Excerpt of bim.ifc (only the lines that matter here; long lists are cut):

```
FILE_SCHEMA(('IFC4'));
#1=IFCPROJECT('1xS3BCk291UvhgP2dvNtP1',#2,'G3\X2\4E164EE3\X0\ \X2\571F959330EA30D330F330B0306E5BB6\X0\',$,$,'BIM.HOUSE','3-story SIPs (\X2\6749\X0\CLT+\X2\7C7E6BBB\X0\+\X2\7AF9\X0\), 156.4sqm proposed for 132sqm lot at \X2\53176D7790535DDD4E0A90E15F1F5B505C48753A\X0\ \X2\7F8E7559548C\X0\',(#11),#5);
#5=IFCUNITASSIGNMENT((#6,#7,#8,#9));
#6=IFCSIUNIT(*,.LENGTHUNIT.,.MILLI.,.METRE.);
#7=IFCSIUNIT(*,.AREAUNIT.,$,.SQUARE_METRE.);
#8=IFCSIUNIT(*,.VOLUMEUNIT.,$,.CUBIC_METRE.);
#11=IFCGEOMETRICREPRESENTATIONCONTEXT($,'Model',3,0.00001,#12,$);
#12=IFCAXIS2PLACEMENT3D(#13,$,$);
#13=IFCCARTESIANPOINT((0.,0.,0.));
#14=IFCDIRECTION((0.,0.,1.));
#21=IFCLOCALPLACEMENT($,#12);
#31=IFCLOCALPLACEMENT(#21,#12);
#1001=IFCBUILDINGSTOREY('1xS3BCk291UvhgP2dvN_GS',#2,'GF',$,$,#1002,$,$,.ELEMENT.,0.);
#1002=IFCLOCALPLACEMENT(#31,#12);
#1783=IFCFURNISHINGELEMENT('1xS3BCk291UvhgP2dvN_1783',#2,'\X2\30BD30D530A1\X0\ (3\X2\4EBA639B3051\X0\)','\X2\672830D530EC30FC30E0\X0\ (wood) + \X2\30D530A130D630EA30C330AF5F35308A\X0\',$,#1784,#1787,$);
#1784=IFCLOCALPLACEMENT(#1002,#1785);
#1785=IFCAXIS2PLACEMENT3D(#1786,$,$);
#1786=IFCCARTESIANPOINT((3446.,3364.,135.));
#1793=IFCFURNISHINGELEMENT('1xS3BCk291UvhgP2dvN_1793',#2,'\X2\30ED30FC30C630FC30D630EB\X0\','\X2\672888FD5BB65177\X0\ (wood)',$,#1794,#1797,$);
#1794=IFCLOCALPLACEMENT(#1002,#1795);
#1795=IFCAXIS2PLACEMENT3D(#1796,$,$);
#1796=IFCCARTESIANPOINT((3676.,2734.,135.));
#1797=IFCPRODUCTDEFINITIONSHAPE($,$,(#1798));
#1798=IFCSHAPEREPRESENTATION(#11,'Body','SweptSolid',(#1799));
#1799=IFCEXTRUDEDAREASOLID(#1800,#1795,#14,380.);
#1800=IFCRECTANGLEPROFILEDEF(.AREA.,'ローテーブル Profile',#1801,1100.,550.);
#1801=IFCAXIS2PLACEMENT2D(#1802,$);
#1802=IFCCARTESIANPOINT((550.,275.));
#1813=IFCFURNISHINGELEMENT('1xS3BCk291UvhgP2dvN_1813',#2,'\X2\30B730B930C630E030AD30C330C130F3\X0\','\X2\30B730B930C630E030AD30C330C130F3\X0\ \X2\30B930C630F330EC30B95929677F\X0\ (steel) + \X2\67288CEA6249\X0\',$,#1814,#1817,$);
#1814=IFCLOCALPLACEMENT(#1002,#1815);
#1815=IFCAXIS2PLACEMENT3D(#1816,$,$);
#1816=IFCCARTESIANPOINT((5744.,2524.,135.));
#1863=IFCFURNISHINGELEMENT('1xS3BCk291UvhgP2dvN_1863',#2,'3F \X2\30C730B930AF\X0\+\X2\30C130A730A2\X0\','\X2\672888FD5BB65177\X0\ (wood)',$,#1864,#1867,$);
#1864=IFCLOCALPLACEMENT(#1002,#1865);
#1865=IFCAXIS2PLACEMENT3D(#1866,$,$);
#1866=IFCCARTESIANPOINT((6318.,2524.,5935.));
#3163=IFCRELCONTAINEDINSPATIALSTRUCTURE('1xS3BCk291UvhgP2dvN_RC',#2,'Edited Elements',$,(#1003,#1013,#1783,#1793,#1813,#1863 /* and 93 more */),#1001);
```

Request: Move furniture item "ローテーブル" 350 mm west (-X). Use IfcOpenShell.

```python
import ifcopenshell
import ifcopenshell.api.geometry
import ifcopenshell.util.placement

model = ifcopenshell.open("bim.ifc")

item = model.by_guid("1xS3BCk291UvhgP2dvN_1793")
matrix = ifcopenshell.util.placement.get_local_placement(item.ObjectPlacement)
matrix[0, 3] -= 350.0
ifcopenshell.api.geometry.edit_object_placement(model, product=item, matrix=matrix, is_si=False)

print(ifcopenshell.util.placement.get_local_placement(item.ObjectPlacement).round(3) + 0.0)

model.write("bim-out.ifc")
```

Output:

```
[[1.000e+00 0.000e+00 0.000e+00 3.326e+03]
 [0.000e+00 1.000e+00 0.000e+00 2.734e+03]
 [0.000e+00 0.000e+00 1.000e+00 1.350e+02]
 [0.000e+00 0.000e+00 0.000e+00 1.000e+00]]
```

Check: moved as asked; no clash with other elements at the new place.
